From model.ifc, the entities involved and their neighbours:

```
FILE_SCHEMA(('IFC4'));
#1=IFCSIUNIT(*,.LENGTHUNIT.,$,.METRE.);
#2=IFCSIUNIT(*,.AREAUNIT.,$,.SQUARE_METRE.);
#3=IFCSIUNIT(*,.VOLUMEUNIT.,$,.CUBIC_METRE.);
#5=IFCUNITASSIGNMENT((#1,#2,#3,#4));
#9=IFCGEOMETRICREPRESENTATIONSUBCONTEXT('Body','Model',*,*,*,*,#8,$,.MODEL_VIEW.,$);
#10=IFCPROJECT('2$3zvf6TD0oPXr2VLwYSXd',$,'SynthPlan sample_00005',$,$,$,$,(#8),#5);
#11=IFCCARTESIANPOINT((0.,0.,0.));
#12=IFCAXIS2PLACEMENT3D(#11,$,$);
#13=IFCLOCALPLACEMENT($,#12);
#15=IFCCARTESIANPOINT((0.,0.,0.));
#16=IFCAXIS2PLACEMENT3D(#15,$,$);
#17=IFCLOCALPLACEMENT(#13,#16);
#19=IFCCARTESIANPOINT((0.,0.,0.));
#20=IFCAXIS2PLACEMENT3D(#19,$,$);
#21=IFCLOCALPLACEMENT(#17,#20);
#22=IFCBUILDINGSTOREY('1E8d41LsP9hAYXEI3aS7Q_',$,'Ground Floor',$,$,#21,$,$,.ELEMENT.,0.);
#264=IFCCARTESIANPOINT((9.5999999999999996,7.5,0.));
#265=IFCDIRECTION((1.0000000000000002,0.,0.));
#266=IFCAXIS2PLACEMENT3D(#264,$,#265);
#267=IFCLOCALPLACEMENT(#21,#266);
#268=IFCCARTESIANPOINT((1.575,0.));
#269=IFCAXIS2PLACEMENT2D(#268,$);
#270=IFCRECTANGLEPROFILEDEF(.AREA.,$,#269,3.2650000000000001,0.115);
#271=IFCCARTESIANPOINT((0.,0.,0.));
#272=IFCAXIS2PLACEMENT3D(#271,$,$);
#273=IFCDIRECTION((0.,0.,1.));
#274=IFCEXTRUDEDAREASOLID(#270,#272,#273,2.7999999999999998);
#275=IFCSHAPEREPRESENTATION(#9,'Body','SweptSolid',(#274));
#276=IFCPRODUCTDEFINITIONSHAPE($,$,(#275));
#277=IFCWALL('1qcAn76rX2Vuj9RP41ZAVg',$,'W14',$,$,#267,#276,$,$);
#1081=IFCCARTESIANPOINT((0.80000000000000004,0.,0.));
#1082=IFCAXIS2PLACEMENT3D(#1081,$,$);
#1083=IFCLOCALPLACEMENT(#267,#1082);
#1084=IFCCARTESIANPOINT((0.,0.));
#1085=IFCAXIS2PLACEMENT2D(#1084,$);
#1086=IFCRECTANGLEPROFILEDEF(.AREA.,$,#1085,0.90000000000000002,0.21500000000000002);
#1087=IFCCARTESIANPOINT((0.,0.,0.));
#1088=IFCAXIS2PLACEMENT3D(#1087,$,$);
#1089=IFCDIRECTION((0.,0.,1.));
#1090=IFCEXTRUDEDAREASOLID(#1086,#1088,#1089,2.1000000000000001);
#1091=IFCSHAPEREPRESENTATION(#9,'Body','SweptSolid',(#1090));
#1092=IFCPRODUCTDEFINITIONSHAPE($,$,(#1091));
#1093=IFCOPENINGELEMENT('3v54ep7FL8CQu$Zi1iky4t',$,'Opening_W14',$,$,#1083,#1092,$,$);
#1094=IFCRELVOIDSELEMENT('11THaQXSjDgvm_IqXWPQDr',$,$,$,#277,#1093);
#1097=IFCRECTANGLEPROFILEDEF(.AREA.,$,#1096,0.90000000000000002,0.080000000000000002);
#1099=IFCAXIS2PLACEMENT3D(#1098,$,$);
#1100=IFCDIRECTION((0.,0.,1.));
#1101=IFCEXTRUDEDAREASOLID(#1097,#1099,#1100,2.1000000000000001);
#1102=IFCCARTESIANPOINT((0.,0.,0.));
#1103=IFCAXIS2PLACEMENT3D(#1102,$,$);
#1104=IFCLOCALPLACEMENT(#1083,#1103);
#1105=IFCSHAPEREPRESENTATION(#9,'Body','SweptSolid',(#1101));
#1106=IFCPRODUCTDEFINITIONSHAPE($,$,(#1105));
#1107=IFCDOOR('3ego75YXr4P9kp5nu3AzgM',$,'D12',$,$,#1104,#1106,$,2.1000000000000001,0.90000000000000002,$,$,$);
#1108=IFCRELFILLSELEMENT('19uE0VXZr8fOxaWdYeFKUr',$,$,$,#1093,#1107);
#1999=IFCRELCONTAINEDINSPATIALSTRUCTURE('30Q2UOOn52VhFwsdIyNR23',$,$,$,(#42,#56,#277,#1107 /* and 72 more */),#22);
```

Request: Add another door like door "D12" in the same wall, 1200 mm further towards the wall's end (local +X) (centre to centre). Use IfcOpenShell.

```python
import ifcopenshell
import ifcopenshell.api.feature
import ifcopenshell.api.geometry
import ifcopenshell.api.root
import ifcopenshell.geom
import ifcopenshell.util.element
import ifcopenshell.util.placement
import ifcopenshell.util.shape

model = ifcopenshell.open("model.ifc")
settings = ifcopenshell.geom.settings()


def volume(element):
    """Net volume in cubic metres, openings subtracted."""
    shape = ifcopenshell.geom.create_shape(settings, element)
    return ifcopenshell.util.shape.get_volume(shape.geometry)


door = model.by_guid("3ego75YXr4P9kp5nu3AzgM")
opening = door.FillsVoids[0].RelatingOpeningElement
wall = opening.VoidsElements[0].RelatingBuildingElement
before = volume(wall)
shift = ifcopenshell.util.placement.get_local_placement(wall.ObjectPlacement)[:3, 0] * 1.2

# copy_class copies the void relationship, type, container and properties, but no geometry.
new_opening = ifcopenshell.api.root.copy_class(model, product=opening)
new_opening.Representation = ifcopenshell.util.element.copy_deep(
    model, opening.Representation, exclude=["IfcGeometricRepresentationContext", "IfcRepresentationMap"]
)
new_door = ifcopenshell.api.root.copy_class(model, product=door)
new_door.Representation = ifcopenshell.util.element.copy_deep(
    model, door.Representation, exclude=["IfcGeometricRepresentationContext", "IfcRepresentationMap"]
)
ifcopenshell.api.feature.add_filling(model, opening=new_opening, element=new_door)

for old, new in ((opening, new_opening), (door, new_door)):
    matrix = ifcopenshell.util.placement.get_local_placement(old.ObjectPlacement)
    matrix[:3, 3] += shift
    ifcopenshell.api.geometry.edit_object_placement(model, product=new, matrix=matrix, is_si=False)

after = volume(wall)

print(f"wall volume {before:.3f} -> {after:.3f} m3")

model.write("model_rev.ifc")
```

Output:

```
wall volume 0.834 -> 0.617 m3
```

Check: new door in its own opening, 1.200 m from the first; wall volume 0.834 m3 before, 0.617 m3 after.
